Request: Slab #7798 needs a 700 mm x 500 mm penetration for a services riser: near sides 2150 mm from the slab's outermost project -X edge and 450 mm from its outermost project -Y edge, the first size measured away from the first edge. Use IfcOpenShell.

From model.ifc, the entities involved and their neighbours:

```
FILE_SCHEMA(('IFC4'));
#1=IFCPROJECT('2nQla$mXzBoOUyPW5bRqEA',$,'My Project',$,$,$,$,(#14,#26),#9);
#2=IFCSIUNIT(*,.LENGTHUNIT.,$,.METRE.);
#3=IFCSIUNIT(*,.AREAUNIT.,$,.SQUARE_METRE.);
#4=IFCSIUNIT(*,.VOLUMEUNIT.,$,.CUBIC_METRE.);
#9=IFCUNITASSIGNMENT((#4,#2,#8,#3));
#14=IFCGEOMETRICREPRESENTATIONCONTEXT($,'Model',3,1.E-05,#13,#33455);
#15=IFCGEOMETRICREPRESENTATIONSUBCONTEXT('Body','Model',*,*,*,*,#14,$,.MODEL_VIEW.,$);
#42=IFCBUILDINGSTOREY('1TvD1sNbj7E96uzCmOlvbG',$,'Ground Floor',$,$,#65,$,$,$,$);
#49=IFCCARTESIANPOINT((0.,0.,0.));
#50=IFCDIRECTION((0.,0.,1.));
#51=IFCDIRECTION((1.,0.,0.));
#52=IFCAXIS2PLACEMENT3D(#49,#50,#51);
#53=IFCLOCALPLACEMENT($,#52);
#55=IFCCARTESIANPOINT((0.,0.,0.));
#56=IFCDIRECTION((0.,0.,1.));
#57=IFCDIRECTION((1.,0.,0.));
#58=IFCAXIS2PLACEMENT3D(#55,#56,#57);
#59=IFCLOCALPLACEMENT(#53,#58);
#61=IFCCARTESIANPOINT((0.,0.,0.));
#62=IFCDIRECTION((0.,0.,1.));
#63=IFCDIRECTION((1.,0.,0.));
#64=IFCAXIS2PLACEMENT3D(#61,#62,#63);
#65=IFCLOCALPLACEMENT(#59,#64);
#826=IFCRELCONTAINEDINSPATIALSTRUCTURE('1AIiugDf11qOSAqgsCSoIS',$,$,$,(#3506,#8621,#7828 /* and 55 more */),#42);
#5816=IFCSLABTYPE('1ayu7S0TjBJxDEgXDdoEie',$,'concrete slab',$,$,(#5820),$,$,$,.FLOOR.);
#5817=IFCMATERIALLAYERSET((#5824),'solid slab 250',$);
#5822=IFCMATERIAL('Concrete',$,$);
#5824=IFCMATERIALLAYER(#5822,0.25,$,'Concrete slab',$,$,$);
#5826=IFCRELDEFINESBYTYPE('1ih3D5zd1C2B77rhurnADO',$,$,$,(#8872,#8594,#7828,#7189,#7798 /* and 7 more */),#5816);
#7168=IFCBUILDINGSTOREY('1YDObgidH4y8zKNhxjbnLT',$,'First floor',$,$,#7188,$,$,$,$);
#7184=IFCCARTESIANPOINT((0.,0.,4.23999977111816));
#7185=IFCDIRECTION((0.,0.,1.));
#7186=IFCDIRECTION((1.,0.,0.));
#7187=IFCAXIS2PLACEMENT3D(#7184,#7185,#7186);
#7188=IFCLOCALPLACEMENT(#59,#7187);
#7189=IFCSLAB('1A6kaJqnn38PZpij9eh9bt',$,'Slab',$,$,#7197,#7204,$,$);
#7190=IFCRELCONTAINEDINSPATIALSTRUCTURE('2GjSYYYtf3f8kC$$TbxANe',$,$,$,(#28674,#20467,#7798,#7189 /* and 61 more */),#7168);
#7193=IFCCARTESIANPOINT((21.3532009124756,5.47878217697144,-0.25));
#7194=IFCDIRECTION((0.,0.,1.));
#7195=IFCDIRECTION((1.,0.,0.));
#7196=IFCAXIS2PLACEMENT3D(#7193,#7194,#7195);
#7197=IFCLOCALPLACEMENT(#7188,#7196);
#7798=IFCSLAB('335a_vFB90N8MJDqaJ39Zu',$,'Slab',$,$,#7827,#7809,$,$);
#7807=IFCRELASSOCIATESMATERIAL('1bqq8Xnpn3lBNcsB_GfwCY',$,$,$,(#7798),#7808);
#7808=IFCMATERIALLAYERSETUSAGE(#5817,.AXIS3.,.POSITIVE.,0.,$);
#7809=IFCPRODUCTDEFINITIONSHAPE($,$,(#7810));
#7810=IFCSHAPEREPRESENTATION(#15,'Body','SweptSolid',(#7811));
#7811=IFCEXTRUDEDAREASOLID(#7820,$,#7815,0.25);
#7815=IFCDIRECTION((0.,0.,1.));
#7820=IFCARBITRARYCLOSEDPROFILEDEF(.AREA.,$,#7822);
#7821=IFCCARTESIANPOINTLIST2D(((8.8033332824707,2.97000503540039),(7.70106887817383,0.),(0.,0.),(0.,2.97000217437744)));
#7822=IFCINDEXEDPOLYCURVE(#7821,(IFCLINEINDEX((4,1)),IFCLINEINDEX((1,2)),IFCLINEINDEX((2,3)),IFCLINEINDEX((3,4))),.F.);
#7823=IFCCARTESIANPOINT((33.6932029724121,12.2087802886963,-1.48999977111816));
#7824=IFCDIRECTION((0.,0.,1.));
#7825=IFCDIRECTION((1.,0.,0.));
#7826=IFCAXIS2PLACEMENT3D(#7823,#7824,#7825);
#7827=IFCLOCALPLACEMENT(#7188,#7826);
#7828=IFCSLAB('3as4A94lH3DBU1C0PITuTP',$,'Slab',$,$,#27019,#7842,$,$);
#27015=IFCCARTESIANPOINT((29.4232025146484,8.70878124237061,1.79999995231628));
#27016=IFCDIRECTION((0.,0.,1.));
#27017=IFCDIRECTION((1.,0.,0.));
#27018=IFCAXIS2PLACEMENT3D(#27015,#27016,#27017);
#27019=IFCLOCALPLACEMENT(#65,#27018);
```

```python
import numpy as np
import ifcopenshell
import ifcopenshell.api.feature
import ifcopenshell.api.geometry
import ifcopenshell.api.root
import ifcopenshell.geom
import ifcopenshell.util.placement
import ifcopenshell.util.representation
import ifcopenshell.util.shape
import ifcopenshell.util.unit

model = ifcopenshell.open("model.ifc")
unit_scale = ifcopenshell.util.unit.calculate_unit_scale(model)
settings = ifcopenshell.geom.settings()


def volume(element):
    """Net volume in cubic metres, openings subtracted."""
    shape = ifcopenshell.geom.create_shape(settings, element)
    return ifcopenshell.util.shape.get_volume(shape.geometry)


slab = model.by_guid("335a_vFB90N8MJDqaJ39Zu")
before = volume(slab)

# Extent in the slab's own axes, in metres. The edges named are its -X and -Y sides.
slab_shape = ifcopenshell.geom.create_shape(settings, slab)
vertices = ifcopenshell.util.shape.get_vertices(slab_shape.geometry)
x_min, y_min, bottom = vertices.min(axis=0)
top = vertices[:, 2].max()

opening = ifcopenshell.api.root.create_entity(model, ifc_class="IfcOpeningElement", name="Services riser opening", predefined_type="OPENING")
context = ifcopenshell.util.representation.get_context(model, "Model", "Body", "MODEL_VIEW")
width, depth = 0.7, 0.5
outline = [(0.0, 0.0), (width, 0.0), (width, depth), (0.0, depth), (0.0, 0.0)]
# Overshoot both faces by 50 mm so the cut is clean.
shape = ifcopenshell.api.geometry.add_slab_representation(
    model, context=context, depth=top - bottom + 0.1, polyline=outline
)
ifcopenshell.api.geometry.assign_representation(model, product=opening, representation=shape)

matrix = ifcopenshell.util.placement.get_local_placement(slab.ObjectPlacement)
matrix[:, 3] = matrix @ np.append(np.array([x_min + 2.15, y_min + 0.45, bottom - 0.05]) / unit_scale, 1.0)
ifcopenshell.api.geometry.edit_object_placement(model, product=opening, matrix=matrix, is_si=False)
ifcopenshell.api.feature.add_feature(model, feature=opening, element=slab)

after = volume(slab)

print(f"slab volume {before:.3f} -> {after:.3f} m3")

model.write("model_updated.ifc")
```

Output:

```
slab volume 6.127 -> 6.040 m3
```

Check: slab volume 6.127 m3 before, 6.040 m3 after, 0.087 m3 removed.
